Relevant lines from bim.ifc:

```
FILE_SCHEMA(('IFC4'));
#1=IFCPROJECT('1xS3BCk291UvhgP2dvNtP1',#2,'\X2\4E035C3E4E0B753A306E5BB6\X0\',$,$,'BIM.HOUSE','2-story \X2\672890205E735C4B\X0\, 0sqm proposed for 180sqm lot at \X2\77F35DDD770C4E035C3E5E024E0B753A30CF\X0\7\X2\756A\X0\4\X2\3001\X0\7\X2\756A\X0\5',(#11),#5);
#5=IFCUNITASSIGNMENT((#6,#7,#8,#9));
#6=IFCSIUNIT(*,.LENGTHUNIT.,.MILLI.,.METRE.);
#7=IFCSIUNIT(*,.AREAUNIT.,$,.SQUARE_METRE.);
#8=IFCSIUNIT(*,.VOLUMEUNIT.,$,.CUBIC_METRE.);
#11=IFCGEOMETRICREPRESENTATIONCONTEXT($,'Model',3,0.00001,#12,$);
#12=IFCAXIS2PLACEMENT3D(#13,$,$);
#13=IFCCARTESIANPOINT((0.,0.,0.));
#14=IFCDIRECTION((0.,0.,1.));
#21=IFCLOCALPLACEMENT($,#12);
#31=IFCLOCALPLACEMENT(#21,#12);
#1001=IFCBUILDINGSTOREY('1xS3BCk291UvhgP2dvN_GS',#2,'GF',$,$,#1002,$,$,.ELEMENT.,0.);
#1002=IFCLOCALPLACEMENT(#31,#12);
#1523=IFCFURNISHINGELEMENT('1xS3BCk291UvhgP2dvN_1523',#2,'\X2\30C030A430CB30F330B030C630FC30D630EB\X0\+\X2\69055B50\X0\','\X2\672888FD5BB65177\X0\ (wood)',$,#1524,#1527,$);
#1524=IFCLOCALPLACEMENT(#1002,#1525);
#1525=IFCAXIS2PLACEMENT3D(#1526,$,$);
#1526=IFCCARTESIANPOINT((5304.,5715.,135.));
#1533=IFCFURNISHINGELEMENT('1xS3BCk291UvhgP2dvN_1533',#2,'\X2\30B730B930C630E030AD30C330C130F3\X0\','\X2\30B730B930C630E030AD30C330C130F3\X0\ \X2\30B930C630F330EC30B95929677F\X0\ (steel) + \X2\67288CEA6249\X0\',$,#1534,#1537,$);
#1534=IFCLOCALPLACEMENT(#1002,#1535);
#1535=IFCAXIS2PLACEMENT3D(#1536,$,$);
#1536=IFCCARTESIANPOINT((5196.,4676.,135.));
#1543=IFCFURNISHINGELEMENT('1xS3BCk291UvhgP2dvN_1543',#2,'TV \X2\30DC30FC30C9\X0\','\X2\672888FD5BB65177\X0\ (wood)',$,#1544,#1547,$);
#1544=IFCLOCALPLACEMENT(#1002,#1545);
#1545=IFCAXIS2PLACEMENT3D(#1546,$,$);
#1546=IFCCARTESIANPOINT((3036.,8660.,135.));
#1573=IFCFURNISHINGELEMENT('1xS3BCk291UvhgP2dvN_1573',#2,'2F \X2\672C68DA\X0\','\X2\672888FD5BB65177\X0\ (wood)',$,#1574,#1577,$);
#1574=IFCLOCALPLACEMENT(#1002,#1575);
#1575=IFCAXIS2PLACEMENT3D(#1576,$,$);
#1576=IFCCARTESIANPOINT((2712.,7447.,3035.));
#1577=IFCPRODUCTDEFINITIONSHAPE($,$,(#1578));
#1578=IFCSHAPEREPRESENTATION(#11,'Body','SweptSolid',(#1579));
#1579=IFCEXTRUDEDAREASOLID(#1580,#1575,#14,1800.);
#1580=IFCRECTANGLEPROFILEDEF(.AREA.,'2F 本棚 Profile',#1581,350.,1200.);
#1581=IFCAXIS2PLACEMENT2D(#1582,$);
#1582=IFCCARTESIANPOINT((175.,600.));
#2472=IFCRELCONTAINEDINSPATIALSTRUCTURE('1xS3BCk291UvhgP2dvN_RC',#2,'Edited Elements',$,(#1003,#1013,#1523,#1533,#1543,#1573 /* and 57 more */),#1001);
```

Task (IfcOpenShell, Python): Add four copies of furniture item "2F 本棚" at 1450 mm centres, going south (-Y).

```python
import numpy as np
import ifcopenshell
import ifcopenshell.api.geometry
import ifcopenshell.api.root
import ifcopenshell.util.element
import ifcopenshell.util.placement
import ifcopenshell.util.unit

model = ifcopenshell.open("bim.ifc")
unit_scale = ifcopenshell.util.unit.calculate_unit_scale(model)


def reuse_history(source, copy):
    """copy_class also copies each property set's owner history, people and application; keep the originals."""
    for rel in copy.IsDefinedBy:
        if rel.is_a("IfcRelDefinesByProperties") and (history := rel.RelatingPropertyDefinition.OwnerHistory):
            rel.RelatingPropertyDefinition.OwnerHistory = source.OwnerHistory
            ifcopenshell.util.element.remove_deep2(model, history)


source = model.by_guid("1xS3BCk291UvhgP2dvN_1573")
base = ifcopenshell.util.placement.get_local_placement(source.ObjectPlacement)
step = np.array([0.0, -1.0, 0.0]) * 1.45 / unit_scale

for i in range(1, 5):
    copy = ifcopenshell.api.root.copy_class(model, product=source)
    copy.Representation = ifcopenshell.util.element.copy_deep(
        model, source.Representation, exclude=["IfcGeometricRepresentationContext", "IfcRepresentationMap"]
    )
    reuse_history(source, copy)
    matrix = base.copy()
    matrix[:3, 3] += i * step
    print("added at", matrix[:3, 3].round(3) + 0.0)
    ifcopenshell.api.geometry.edit_object_placement(model, product=copy, matrix=matrix, is_si=False)

model.write("bim-out.ifc")
```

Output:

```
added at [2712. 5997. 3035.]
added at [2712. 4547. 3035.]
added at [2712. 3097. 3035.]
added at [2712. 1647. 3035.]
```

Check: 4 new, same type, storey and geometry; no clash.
